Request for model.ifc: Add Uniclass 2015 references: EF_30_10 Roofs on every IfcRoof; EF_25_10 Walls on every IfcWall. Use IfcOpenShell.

First a look at what the model holds.

```python
import ifcopenshell

model = ifcopenshell.open("model.ifc")
print(model.schema)
print("classifications:", [c.Name for c in model.by_type("IfcClassification")])
for ifc_class in ("IfcDoor", "IfcRoof", "IfcStair", "IfcWall", "IfcWindow"):
    print(ifc_class, len(model.by_type(ifc_class)))
```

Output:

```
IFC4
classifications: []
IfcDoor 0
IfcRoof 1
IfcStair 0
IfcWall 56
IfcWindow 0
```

```python
import ifcopenshell
import ifcopenshell.api.classification

model = ifcopenshell.open("model.ifc")

system = ifcopenshell.api.classification.add_classification(model, classification="Uniclass 2015")

codes = {
    "IfcRoof": ("EF_30_10", "Roofs"),
    "IfcWall": ("EF_25_10", "Walls"),
}
for ifc_class, (code, name) in codes.items():
    products = model.by_type(ifc_class)
    ifcopenshell.api.classification.add_reference(
        model, products=products, classification=system, identification=code, name=name
    )
    print(code, len(products))

model.write("model_rev.ifc")
```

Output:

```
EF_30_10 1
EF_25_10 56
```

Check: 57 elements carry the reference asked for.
